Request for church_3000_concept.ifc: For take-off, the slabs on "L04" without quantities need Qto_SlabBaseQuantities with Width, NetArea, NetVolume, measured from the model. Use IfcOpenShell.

First a look at what the model holds.

```python
import ifcopenshell
import ifcopenshell.util.element
import ifcopenshell.util.unit

model = ifcopenshell.open("church_3000_concept.ifc")
print(model.schema)
for unit_type in ("LENGTHUNIT", "AREAUNIT", "VOLUMEUNIT"):
    print(unit_type, ifcopenshell.util.unit.calculate_unit_scale(model, unit_type))
storey = next(s for s in model.by_type("IfcBuildingStorey") if s.Name == "L04")
slabs = [e for e in ifcopenshell.util.element.get_decomposition(storey) if e.is_a("IfcSlab")]
for e in sorted(slabs, key=lambda e: e.id()):
    print(e.id(), e.is_a(), e.Name, list(ifcopenshell.util.element.get_psets(e, qtos_only=True)), sep=" | ")
```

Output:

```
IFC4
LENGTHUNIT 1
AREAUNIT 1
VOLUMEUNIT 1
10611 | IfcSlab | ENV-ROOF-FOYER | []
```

```python
import ifcopenshell
import ifcopenshell.api.pset
import ifcopenshell.geom
import ifcopenshell.util.element
import ifcopenshell.util.shape
import ifcopenshell.util.unit

model = ifcopenshell.open("church_3000_concept.ifc")
unit_scale = ifcopenshell.util.unit.calculate_unit_scale(model)
area_scale = ifcopenshell.util.unit.calculate_unit_scale(model, "AREAUNIT")
volume_scale = ifcopenshell.util.unit.calculate_unit_scale(model, "VOLUMEUNIT")
settings = ifcopenshell.geom.settings()

storey = next(s for s in model.by_type("IfcBuildingStorey") if s.Name == "L04")
slabs = [e for e in ifcopenshell.util.element.get_decomposition(storey) if e.is_a("IfcSlab")]

for e in sorted(slabs, key=lambda e: e.id()):
    if ifcopenshell.util.element.get_psets(e, qtos_only=True, should_inherit=False):
        continue
    # Geometry comes back in metres, in the element's own axes.
    shape = ifcopenshell.geom.create_shape(settings, e)
    values = {
        "Width": ifcopenshell.util.shape.get_z(shape.geometry) / unit_scale,
        "NetArea": ifcopenshell.util.shape.get_footprint_area(shape.geometry) / area_scale,
        "NetVolume": ifcopenshell.util.shape.get_volume(shape.geometry) / volume_scale,
    }
    qto = ifcopenshell.api.pset.add_qto(model, product=e, name="Qto_SlabBaseQuantities")
    ifcopenshell.api.pset.edit_qto(model, qto=qto, properties=values)
    print(e.id(), {k: round(v, 3) for k, v in values.items()})

model.write("church_3000_concept_edited.ifc")
```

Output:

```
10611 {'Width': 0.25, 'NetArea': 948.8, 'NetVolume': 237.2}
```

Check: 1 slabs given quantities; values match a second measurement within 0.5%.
